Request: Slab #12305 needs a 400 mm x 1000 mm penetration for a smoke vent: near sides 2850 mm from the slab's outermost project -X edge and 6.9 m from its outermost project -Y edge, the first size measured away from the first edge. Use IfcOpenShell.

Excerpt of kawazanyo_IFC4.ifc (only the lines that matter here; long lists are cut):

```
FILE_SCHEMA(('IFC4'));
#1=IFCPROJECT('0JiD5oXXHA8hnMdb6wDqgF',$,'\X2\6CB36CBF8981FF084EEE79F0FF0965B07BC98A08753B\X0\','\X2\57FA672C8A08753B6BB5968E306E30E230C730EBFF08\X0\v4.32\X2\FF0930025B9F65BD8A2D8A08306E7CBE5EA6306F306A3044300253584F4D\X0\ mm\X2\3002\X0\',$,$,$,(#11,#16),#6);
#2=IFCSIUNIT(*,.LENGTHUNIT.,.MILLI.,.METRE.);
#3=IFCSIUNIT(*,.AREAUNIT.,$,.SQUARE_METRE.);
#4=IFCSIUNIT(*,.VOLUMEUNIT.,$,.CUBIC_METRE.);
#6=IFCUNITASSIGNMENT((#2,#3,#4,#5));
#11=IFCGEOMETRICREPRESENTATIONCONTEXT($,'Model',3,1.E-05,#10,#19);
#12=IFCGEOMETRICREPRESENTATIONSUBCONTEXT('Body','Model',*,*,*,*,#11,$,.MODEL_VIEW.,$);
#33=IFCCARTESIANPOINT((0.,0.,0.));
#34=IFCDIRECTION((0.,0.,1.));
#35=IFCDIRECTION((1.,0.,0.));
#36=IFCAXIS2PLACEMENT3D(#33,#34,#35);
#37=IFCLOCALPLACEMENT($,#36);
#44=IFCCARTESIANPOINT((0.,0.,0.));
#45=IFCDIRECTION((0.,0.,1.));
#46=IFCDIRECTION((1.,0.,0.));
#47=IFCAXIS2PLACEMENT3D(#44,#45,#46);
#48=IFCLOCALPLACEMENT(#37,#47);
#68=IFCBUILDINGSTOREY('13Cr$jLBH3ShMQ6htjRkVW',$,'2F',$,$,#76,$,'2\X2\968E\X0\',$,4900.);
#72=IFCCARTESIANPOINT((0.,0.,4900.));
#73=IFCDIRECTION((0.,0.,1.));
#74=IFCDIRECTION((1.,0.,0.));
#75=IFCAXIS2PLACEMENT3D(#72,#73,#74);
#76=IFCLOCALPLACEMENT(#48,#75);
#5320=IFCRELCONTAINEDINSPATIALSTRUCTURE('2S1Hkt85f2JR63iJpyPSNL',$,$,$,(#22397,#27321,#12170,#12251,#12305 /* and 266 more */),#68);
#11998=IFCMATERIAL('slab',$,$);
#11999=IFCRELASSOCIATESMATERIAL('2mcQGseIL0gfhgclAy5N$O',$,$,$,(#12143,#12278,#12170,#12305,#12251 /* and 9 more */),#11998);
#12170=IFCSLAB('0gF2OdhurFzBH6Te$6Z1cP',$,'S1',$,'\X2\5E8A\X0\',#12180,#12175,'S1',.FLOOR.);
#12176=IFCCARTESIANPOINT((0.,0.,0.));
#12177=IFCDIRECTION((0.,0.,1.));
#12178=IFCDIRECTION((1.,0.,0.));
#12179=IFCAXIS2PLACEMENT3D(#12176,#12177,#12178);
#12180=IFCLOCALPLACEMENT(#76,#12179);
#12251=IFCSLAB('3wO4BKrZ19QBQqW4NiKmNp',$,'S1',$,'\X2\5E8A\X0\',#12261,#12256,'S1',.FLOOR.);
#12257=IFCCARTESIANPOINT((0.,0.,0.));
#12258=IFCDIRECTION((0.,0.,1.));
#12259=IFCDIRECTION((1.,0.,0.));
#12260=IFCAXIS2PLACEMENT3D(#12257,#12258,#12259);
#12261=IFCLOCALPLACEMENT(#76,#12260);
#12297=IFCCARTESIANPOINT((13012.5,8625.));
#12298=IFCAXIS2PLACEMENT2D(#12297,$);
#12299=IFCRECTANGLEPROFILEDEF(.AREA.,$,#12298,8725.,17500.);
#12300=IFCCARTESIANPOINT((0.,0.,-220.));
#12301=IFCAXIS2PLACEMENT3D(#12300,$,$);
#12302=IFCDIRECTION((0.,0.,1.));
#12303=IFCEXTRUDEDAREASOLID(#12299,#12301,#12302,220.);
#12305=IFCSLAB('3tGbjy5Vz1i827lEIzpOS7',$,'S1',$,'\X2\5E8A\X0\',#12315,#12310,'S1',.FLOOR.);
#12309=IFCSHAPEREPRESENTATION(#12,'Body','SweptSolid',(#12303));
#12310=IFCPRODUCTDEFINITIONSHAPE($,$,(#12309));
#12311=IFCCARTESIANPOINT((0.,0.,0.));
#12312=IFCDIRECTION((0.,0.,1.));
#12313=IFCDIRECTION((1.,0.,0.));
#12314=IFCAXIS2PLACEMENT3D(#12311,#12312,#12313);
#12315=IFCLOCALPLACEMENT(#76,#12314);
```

```python
import numpy as np
import ifcopenshell
import ifcopenshell.api.feature
import ifcopenshell.api.geometry
import ifcopenshell.api.root
import ifcopenshell.geom
import ifcopenshell.util.placement
import ifcopenshell.util.representation
import ifcopenshell.util.shape
import ifcopenshell.util.unit

model = ifcopenshell.open("kawazanyo_IFC4.ifc")
unit_scale = ifcopenshell.util.unit.calculate_unit_scale(model)
settings = ifcopenshell.geom.settings()


def volume(element):
    """Net volume in cubic metres, openings subtracted."""
    shape = ifcopenshell.geom.create_shape(settings, element)
    return ifcopenshell.util.shape.get_volume(shape.geometry)


slab = model.by_guid("3tGbjy5Vz1i827lEIzpOS7")
before = volume(slab)

# Extent in the slab's own axes, in metres. The edges named are its -X and -Y sides.
slab_shape = ifcopenshell.geom.create_shape(settings, slab)
vertices = ifcopenshell.util.shape.get_vertices(slab_shape.geometry)
x_min, y_min, bottom = vertices.min(axis=0)
top = vertices[:, 2].max()

opening = ifcopenshell.api.root.create_entity(model, ifc_class="IfcOpeningElement", name="Smoke vent opening", predefined_type="OPENING")
context = ifcopenshell.util.representation.get_context(model, "Model", "Body", "MODEL_VIEW")
width, depth = 0.4, 1
outline = [(0.0, 0.0), (width, 0.0), (width, depth), (0.0, depth), (0.0, 0.0)]
# Overshoot both faces by 50 mm so the cut is clean.
shape = ifcopenshell.api.geometry.add_slab_representation(
    model, context=context, depth=top - bottom + 0.1, polyline=outline
)
ifcopenshell.api.geometry.assign_representation(model, product=opening, representation=shape)

matrix = ifcopenshell.util.placement.get_local_placement(slab.ObjectPlacement)
matrix[:, 3] = matrix @ np.append(np.array([x_min + 2.85, y_min + 6.9, bottom - 0.05]) / unit_scale, 1.0)
ifcopenshell.api.geometry.edit_object_placement(model, product=opening, matrix=matrix, is_si=False)
ifcopenshell.api.feature.add_feature(model, feature=opening, element=slab)

after = volume(slab)

print(f"slab volume {before:.3f} -> {after:.3f} m3")

model.write("kawazanyo_IFC4_v2.ifc")
```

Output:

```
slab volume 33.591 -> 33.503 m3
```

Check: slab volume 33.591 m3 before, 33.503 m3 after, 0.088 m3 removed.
